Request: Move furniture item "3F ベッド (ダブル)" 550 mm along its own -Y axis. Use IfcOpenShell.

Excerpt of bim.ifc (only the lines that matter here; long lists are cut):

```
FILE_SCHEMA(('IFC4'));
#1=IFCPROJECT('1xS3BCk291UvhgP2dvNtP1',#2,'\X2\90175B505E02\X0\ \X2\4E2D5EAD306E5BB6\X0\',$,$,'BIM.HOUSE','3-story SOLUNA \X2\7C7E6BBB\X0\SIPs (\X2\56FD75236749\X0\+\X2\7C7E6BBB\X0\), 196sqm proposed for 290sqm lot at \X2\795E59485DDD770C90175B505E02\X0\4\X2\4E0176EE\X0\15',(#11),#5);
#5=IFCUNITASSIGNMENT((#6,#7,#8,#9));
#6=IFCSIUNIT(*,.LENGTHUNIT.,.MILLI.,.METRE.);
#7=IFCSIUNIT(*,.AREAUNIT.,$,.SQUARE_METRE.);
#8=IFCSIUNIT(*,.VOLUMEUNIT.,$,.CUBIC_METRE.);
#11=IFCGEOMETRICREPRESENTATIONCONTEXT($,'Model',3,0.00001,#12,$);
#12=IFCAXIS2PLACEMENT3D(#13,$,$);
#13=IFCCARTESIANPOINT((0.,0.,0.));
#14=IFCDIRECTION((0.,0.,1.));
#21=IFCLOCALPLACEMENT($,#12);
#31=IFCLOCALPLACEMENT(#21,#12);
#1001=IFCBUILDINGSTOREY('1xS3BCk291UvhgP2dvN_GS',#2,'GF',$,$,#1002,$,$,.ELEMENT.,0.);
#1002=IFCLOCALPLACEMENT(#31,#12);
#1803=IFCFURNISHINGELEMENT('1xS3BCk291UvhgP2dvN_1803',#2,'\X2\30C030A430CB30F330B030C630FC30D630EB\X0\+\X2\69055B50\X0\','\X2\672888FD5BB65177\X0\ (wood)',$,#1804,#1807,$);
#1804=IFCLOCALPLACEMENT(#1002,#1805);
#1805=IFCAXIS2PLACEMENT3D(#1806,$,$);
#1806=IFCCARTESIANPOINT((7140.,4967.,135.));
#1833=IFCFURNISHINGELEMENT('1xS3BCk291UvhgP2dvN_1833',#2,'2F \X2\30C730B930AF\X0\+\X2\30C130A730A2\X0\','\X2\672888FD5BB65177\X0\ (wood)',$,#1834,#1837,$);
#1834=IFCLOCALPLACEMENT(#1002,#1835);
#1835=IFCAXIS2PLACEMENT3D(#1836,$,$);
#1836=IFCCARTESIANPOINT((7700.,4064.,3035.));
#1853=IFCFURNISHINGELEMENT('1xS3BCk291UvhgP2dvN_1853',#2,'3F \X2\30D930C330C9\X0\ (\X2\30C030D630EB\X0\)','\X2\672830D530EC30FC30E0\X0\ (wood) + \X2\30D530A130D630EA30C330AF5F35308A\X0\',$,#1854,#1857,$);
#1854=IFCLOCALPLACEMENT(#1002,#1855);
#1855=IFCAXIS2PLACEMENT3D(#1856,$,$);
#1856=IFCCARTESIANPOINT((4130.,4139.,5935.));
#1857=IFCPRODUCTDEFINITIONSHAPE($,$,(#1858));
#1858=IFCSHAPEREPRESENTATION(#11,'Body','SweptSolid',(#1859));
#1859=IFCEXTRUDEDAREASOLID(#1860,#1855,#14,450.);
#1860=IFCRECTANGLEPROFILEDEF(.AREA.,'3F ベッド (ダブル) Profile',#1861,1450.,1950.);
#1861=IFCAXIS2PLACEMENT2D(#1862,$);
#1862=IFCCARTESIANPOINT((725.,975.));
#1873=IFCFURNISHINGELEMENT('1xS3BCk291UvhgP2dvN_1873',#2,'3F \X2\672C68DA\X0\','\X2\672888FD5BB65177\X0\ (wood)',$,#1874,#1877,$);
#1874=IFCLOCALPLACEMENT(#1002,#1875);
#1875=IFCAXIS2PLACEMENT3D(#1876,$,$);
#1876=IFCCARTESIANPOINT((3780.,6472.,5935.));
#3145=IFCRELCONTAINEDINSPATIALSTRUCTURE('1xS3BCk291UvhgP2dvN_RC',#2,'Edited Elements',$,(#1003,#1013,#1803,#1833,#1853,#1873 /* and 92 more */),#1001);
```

```python
import ifcopenshell
import ifcopenshell.api.geometry
import ifcopenshell.util.placement

model = ifcopenshell.open("bim.ifc")

item = model.by_guid("1xS3BCk291UvhgP2dvN_1853")
matrix = ifcopenshell.util.placement.get_local_placement(item.ObjectPlacement)
matrix[:3, 3] -= matrix[:3, 1] * 550.0
ifcopenshell.api.geometry.edit_object_placement(model, product=item, matrix=matrix, is_si=False)

print(ifcopenshell.util.placement.get_local_placement(item.ObjectPlacement).round(3) + 0.0)

model.write("bim_updated.ifc")
```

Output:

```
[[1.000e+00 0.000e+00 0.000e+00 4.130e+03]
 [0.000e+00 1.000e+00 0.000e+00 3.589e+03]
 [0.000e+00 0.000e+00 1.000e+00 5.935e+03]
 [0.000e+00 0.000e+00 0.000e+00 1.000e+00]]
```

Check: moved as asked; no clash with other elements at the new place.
